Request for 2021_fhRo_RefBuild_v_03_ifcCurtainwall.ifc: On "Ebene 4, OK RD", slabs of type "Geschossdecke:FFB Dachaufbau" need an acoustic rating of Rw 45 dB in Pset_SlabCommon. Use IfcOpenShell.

First a look at what the model holds.

```python
import ifcopenshell
import ifcopenshell.util.element

model = ifcopenshell.open("2021_fhRo_RefBuild_v_03_ifcCurtainwall.ifc")
print(model.schema)
storey = next(s for s in model.by_type("IfcBuildingStorey") if s.Name == "Ebene 4, OK RD")
slabs = [e for e in ifcopenshell.util.element.get_decomposition(storey) if e.is_a("IfcSlab")]
seen = {}
for e in slabs:
    element_type = ifcopenshell.util.element.get_type(e)
    key = (element_type.Name if element_type != e and element_type else None, ifcopenshell.util.element.get_pset(e, "Pset_SlabCommon", "AcousticRating"))
    seen[key] = seen.get(key, 0) + 1
for (name, value), count in sorted(seen.items(), key=str):
    print(count, "x", name, "|", value)
```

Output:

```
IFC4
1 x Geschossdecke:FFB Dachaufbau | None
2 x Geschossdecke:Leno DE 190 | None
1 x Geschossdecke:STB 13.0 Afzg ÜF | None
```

```python
import ifcopenshell
import ifcopenshell.api.pset
import ifcopenshell.util.element

model = ifcopenshell.open("2021_fhRo_RefBuild_v_03_ifcCurtainwall.ifc")

storey = next(s for s in model.by_type("IfcBuildingStorey") if s.Name == "Ebene 4, OK RD")
slabs = [e for e in ifcopenshell.util.element.get_decomposition(storey) if e.is_a("IfcSlab")]

count = 0
for e in slabs:
    element_type = ifcopenshell.util.element.get_type(e)
    if element_type in (None, e) or element_type.Name != "Geschossdecke:FFB Dachaufbau":
        continue
    # add_pset returns the element's existing set when there is one.
    pset = ifcopenshell.api.pset.add_pset(model, product=e, name="Pset_SlabCommon")
    ifcopenshell.api.pset.edit_pset(model, pset=pset, properties={"AcousticRating": "Rw 45 dB"})
    count += 1

print(count, "slabs updated")

model.write("2021_fhRo_RefBuild_v_03_ifcCurtainwall_rev.ifc")
```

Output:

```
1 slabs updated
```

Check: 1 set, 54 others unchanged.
